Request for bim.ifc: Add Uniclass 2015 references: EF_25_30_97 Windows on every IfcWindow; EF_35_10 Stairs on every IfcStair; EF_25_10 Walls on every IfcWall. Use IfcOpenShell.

First a look at what the model holds.

```python
import ifcopenshell

model = ifcopenshell.open("bim.ifc")
print(model.schema)
print("classifications:", [c.Name for c in model.by_type("IfcClassification")])
for ifc_class in ("IfcDoor", "IfcRoof", "IfcStair", "IfcWall", "IfcWindow"):
    print(ifc_class, len(model.by_type(ifc_class)))
```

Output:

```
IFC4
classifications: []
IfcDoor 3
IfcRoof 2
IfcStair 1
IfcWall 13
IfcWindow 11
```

```python
import ifcopenshell
import ifcopenshell.api.classification

model = ifcopenshell.open("bim.ifc")

system = ifcopenshell.api.classification.add_classification(model, classification="Uniclass 2015")

codes = {
    "IfcWindow": ("EF_25_30_97", "Windows"),
    "IfcStair": ("EF_35_10", "Stairs"),
    "IfcWall": ("EF_25_10", "Walls"),
}
for ifc_class, (code, name) in codes.items():
    products = model.by_type(ifc_class)
    ifcopenshell.api.classification.add_reference(
        model, products=products, classification=system, identification=code, name=name
    )
    print(code, len(products))

model.write("bim_v2.ifc")
```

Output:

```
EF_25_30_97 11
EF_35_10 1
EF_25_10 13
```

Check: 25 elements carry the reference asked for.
